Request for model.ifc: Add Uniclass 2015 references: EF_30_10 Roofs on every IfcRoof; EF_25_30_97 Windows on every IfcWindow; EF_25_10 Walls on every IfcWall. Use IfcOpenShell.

First a look at what the model holds.

```python
import ifcopenshell

model = ifcopenshell.open("model.ifc")
print(model.schema)
print("classifications:", [c.Name for c in model.by_type("IfcClassification")])
for ifc_class in ("IfcDoor", "IfcRoof", "IfcStair", "IfcWall", "IfcWindow"):
    print(ifc_class, len(model.by_type(ifc_class)))
```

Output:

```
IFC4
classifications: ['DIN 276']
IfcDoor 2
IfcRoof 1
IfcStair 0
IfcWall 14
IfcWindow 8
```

```python
import ifcopenshell
import ifcopenshell.api.classification

model = ifcopenshell.open("model.ifc")

system = ifcopenshell.api.classification.add_classification(model, classification="Uniclass 2015")

codes = {
    "IfcRoof": ("EF_30_10", "Roofs"),
    "IfcWindow": ("EF_25_30_97", "Windows"),
    "IfcWall": ("EF_25_10", "Walls"),
}
for ifc_class, (code, name) in codes.items():
    products = model.by_type(ifc_class)
    ifcopenshell.api.classification.add_reference(
        model, products=products, classification=system, identification=code, name=name
    )
    print(code, len(products))

model.write("model_edited.ifc")
```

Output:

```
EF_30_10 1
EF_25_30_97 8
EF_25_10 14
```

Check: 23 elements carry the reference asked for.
